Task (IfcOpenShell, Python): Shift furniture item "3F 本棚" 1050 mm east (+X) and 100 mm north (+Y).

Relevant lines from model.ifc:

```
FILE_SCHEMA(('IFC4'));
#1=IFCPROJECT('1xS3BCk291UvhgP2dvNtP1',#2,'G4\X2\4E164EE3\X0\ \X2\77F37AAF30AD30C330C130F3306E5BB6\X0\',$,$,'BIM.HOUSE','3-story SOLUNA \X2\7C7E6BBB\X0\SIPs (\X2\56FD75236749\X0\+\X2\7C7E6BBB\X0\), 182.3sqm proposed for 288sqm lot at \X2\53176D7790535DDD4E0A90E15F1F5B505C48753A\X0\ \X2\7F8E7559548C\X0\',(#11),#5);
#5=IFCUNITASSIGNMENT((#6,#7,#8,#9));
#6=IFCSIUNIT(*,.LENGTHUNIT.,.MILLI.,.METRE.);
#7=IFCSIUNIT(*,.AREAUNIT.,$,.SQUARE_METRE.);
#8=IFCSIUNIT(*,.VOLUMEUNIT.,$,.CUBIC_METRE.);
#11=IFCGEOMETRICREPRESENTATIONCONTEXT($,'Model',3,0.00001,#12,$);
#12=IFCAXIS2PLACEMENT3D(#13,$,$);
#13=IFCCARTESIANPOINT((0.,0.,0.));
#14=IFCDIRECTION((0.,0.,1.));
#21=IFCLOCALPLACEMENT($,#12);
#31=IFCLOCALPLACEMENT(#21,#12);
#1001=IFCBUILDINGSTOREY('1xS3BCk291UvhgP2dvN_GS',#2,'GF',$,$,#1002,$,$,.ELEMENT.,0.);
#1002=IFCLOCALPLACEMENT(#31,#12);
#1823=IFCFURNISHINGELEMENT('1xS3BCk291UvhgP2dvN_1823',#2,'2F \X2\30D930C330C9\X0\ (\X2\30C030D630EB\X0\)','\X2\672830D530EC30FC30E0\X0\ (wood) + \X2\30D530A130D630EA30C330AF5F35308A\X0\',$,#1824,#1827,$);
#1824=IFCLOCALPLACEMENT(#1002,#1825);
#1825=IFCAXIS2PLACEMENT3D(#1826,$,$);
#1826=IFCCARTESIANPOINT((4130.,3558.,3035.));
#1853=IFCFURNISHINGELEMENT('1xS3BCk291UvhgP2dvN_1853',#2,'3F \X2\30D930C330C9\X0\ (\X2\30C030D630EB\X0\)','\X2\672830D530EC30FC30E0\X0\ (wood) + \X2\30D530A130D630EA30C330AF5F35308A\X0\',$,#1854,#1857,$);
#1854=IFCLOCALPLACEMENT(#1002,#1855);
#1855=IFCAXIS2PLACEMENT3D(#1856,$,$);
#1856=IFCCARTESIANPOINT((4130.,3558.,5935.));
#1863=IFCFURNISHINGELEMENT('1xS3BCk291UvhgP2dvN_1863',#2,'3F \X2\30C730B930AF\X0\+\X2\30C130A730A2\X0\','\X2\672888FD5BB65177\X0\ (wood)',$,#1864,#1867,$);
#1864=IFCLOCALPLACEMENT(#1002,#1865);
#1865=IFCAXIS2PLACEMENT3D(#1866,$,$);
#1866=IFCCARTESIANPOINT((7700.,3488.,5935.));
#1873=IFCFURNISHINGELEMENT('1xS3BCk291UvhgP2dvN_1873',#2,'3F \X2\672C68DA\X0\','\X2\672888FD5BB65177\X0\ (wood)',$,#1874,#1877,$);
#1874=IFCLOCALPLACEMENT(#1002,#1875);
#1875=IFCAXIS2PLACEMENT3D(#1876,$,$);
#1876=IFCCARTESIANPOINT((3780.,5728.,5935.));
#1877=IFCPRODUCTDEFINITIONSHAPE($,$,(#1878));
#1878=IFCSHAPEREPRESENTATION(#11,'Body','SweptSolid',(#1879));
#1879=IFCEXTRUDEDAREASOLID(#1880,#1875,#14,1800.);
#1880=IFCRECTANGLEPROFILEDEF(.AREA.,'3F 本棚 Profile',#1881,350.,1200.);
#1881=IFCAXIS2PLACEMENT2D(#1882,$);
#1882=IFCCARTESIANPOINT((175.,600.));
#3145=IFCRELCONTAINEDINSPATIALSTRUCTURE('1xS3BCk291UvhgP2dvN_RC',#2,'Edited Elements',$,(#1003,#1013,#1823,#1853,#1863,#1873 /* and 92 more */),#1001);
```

```python
import ifcopenshell
import ifcopenshell.api.geometry
import ifcopenshell.util.placement
import ifcopenshell.util.unit

model = ifcopenshell.open("model.ifc")
unit_scale = ifcopenshell.util.unit.calculate_unit_scale(model)

item = model.by_guid("1xS3BCk291UvhgP2dvN_1873")
matrix = ifcopenshell.util.placement.get_local_placement(item.ObjectPlacement)
matrix[0, 3] += 1.05 / unit_scale
matrix[1, 3] += 0.1 / unit_scale
ifcopenshell.api.geometry.edit_object_placement(model, product=item, matrix=matrix, is_si=False)

print(ifcopenshell.util.placement.get_local_placement(item.ObjectPlacement).round(3) + 0.0)

model.write("model_edited.ifc")
```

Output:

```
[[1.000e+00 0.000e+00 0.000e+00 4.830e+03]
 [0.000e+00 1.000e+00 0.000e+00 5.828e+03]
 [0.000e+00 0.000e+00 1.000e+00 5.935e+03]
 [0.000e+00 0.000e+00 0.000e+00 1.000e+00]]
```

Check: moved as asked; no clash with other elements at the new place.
